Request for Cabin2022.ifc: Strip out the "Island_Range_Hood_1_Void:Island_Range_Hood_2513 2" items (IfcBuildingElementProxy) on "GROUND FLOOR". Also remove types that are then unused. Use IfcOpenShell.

First a look at what the model holds.

```python
import ifcopenshell
import ifcopenshell.util.element

model = ifcopenshell.open("Cabin2022.ifc")
print(model.schema)
storey = next(s for s in model.by_type("IfcBuildingStorey") if s.Name == "GROUND FLOOR")
proxies = [e for e in ifcopenshell.util.element.get_decomposition(storey) if e.is_a("IfcBuildingElementProxy")]
seen = {}
for e in proxies:
    element_type = ifcopenshell.util.element.get_type(e)
    name = element_type.Name if element_type not in (None, e) else None
    seen[name] = seen.get(name, 0) + 1
for name, count in sorted(seen.items(), key=str):
    print(count, "x", name)
```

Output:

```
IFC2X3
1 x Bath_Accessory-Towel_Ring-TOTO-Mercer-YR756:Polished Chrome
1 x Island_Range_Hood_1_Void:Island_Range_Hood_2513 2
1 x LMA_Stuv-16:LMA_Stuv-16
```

```python
import ifcopenshell
import ifcopenshell.api.root
import ifcopenshell.util.element

model = ifcopenshell.open("Cabin2022.ifc")

storey = next(s for s in model.by_type("IfcBuildingStorey") if s.Name == "GROUND FLOOR")
proxies = [e for e in ifcopenshell.util.element.get_decomposition(storey) if e.is_a("IfcBuildingElementProxy")]
targets = [e for e in proxies if (t := ifcopenshell.util.element.get_type(e)) not in (None, e) and t.Name == "Island_Range_Hood_1_Void:Island_Range_Hood_2513 2"]
types = {ifcopenshell.util.element.get_type(e) for e in targets} - {None, *targets}

for e in targets:
    ifcopenshell.api.root.remove_product(model, product=e)
print(len(targets), "removed")

unused = [t for t in types if not ifcopenshell.util.element.get_types(t)]
for t in unused:
    ifcopenshell.api.root.remove_product(model, product=t)
print(len(unused), "unused types removed")

model.write("Cabin2022_v2.ifc")
```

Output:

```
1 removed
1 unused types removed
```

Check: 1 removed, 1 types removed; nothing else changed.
